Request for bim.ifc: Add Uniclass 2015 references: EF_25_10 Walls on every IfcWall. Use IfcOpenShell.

First a look at what the model holds.

```python
import ifcopenshell

model = ifcopenshell.open("bim.ifc")
print(model.schema)
print("classifications:", [c.Name for c in model.by_type("IfcClassification")])
for ifc_class in ("IfcDoor", "IfcRoof", "IfcStair", "IfcWall", "IfcWindow"):
    print(ifc_class, len(model.by_type(ifc_class)))
```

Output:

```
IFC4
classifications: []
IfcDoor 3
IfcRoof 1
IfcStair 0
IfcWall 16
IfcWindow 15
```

```python
import ifcopenshell
import ifcopenshell.api.classification

model = ifcopenshell.open("bim.ifc")

system = ifcopenshell.api.classification.add_classification(model, classification="Uniclass 2015")

codes = {
    "IfcWall": ("EF_25_10", "Walls"),
}
for ifc_class, (code, name) in codes.items():
    products = model.by_type(ifc_class)
    ifcopenshell.api.classification.add_reference(
        model, products=products, classification=system, identification=code, name=name
    )
    print(code, len(products))

model.write("bim-out.ifc")
```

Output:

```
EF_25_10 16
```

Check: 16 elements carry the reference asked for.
